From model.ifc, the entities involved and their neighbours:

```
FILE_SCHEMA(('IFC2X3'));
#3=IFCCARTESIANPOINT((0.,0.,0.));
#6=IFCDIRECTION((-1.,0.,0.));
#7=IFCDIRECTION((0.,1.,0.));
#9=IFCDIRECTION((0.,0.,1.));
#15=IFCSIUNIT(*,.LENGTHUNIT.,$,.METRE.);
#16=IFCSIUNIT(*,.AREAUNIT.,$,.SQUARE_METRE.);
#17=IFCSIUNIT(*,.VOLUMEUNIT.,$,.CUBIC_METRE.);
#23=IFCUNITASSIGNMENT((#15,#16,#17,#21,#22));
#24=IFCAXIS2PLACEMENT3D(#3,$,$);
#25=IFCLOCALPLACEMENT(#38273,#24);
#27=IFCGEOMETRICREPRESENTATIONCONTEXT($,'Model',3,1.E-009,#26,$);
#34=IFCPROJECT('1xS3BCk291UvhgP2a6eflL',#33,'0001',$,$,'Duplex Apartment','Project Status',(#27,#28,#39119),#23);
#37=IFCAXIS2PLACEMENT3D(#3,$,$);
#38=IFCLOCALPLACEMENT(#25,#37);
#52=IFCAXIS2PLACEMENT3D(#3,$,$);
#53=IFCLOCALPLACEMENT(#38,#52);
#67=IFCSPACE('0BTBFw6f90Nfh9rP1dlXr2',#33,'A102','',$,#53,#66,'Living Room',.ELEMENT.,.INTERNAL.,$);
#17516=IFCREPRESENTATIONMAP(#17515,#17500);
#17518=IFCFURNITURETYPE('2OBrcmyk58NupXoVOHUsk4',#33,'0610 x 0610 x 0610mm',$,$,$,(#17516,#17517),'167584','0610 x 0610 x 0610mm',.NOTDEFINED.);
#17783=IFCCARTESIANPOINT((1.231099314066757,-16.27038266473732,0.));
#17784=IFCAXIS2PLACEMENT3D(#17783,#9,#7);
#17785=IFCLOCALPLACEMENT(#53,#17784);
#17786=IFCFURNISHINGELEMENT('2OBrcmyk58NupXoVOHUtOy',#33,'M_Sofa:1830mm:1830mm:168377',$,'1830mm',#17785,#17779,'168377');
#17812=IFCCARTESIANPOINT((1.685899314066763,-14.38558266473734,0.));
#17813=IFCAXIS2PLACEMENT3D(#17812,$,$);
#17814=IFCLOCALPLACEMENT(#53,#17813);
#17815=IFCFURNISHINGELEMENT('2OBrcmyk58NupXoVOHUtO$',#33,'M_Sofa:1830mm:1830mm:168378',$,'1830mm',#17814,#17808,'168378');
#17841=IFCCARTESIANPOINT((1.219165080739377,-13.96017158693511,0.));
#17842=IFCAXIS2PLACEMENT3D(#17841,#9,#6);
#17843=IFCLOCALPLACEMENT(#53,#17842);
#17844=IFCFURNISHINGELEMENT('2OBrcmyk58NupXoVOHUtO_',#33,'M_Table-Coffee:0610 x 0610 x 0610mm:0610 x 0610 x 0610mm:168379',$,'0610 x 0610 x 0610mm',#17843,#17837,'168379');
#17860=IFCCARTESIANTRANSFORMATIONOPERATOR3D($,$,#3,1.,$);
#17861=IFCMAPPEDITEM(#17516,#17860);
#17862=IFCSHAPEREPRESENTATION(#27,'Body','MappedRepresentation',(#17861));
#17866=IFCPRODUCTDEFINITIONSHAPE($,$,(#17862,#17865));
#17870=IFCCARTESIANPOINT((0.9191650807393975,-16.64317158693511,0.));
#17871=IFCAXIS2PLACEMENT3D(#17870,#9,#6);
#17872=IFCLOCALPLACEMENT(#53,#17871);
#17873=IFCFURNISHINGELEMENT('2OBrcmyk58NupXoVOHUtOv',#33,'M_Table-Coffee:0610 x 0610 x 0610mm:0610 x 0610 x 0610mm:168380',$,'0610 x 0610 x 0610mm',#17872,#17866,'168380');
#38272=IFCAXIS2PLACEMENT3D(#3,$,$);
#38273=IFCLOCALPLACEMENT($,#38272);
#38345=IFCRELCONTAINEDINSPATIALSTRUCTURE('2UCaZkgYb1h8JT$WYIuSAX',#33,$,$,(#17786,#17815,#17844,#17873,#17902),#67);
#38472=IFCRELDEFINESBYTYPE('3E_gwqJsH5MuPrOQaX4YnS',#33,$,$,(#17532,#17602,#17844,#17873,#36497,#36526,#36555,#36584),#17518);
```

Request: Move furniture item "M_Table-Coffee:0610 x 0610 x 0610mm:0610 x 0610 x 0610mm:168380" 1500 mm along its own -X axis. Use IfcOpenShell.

```python
import ifcopenshell
import ifcopenshell.api.geometry
import ifcopenshell.util.placement
import ifcopenshell.util.unit

model = ifcopenshell.open("model.ifc")
unit_scale = ifcopenshell.util.unit.calculate_unit_scale(model)

item = model.by_id(17873)
matrix = ifcopenshell.util.placement.get_local_placement(item.ObjectPlacement)
matrix[:3, 3] -= matrix[:3, 0] * 1.5 / unit_scale
ifcopenshell.api.geometry.edit_object_placement(model, product=item, matrix=matrix, is_si=False)

print(ifcopenshell.util.placement.get_local_placement(item.ObjectPlacement).round(3) + 0.0)

model.write("model_edited.ifc")
```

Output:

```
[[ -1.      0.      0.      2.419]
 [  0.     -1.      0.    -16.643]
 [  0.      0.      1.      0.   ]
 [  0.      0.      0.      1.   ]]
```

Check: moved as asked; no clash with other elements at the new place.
